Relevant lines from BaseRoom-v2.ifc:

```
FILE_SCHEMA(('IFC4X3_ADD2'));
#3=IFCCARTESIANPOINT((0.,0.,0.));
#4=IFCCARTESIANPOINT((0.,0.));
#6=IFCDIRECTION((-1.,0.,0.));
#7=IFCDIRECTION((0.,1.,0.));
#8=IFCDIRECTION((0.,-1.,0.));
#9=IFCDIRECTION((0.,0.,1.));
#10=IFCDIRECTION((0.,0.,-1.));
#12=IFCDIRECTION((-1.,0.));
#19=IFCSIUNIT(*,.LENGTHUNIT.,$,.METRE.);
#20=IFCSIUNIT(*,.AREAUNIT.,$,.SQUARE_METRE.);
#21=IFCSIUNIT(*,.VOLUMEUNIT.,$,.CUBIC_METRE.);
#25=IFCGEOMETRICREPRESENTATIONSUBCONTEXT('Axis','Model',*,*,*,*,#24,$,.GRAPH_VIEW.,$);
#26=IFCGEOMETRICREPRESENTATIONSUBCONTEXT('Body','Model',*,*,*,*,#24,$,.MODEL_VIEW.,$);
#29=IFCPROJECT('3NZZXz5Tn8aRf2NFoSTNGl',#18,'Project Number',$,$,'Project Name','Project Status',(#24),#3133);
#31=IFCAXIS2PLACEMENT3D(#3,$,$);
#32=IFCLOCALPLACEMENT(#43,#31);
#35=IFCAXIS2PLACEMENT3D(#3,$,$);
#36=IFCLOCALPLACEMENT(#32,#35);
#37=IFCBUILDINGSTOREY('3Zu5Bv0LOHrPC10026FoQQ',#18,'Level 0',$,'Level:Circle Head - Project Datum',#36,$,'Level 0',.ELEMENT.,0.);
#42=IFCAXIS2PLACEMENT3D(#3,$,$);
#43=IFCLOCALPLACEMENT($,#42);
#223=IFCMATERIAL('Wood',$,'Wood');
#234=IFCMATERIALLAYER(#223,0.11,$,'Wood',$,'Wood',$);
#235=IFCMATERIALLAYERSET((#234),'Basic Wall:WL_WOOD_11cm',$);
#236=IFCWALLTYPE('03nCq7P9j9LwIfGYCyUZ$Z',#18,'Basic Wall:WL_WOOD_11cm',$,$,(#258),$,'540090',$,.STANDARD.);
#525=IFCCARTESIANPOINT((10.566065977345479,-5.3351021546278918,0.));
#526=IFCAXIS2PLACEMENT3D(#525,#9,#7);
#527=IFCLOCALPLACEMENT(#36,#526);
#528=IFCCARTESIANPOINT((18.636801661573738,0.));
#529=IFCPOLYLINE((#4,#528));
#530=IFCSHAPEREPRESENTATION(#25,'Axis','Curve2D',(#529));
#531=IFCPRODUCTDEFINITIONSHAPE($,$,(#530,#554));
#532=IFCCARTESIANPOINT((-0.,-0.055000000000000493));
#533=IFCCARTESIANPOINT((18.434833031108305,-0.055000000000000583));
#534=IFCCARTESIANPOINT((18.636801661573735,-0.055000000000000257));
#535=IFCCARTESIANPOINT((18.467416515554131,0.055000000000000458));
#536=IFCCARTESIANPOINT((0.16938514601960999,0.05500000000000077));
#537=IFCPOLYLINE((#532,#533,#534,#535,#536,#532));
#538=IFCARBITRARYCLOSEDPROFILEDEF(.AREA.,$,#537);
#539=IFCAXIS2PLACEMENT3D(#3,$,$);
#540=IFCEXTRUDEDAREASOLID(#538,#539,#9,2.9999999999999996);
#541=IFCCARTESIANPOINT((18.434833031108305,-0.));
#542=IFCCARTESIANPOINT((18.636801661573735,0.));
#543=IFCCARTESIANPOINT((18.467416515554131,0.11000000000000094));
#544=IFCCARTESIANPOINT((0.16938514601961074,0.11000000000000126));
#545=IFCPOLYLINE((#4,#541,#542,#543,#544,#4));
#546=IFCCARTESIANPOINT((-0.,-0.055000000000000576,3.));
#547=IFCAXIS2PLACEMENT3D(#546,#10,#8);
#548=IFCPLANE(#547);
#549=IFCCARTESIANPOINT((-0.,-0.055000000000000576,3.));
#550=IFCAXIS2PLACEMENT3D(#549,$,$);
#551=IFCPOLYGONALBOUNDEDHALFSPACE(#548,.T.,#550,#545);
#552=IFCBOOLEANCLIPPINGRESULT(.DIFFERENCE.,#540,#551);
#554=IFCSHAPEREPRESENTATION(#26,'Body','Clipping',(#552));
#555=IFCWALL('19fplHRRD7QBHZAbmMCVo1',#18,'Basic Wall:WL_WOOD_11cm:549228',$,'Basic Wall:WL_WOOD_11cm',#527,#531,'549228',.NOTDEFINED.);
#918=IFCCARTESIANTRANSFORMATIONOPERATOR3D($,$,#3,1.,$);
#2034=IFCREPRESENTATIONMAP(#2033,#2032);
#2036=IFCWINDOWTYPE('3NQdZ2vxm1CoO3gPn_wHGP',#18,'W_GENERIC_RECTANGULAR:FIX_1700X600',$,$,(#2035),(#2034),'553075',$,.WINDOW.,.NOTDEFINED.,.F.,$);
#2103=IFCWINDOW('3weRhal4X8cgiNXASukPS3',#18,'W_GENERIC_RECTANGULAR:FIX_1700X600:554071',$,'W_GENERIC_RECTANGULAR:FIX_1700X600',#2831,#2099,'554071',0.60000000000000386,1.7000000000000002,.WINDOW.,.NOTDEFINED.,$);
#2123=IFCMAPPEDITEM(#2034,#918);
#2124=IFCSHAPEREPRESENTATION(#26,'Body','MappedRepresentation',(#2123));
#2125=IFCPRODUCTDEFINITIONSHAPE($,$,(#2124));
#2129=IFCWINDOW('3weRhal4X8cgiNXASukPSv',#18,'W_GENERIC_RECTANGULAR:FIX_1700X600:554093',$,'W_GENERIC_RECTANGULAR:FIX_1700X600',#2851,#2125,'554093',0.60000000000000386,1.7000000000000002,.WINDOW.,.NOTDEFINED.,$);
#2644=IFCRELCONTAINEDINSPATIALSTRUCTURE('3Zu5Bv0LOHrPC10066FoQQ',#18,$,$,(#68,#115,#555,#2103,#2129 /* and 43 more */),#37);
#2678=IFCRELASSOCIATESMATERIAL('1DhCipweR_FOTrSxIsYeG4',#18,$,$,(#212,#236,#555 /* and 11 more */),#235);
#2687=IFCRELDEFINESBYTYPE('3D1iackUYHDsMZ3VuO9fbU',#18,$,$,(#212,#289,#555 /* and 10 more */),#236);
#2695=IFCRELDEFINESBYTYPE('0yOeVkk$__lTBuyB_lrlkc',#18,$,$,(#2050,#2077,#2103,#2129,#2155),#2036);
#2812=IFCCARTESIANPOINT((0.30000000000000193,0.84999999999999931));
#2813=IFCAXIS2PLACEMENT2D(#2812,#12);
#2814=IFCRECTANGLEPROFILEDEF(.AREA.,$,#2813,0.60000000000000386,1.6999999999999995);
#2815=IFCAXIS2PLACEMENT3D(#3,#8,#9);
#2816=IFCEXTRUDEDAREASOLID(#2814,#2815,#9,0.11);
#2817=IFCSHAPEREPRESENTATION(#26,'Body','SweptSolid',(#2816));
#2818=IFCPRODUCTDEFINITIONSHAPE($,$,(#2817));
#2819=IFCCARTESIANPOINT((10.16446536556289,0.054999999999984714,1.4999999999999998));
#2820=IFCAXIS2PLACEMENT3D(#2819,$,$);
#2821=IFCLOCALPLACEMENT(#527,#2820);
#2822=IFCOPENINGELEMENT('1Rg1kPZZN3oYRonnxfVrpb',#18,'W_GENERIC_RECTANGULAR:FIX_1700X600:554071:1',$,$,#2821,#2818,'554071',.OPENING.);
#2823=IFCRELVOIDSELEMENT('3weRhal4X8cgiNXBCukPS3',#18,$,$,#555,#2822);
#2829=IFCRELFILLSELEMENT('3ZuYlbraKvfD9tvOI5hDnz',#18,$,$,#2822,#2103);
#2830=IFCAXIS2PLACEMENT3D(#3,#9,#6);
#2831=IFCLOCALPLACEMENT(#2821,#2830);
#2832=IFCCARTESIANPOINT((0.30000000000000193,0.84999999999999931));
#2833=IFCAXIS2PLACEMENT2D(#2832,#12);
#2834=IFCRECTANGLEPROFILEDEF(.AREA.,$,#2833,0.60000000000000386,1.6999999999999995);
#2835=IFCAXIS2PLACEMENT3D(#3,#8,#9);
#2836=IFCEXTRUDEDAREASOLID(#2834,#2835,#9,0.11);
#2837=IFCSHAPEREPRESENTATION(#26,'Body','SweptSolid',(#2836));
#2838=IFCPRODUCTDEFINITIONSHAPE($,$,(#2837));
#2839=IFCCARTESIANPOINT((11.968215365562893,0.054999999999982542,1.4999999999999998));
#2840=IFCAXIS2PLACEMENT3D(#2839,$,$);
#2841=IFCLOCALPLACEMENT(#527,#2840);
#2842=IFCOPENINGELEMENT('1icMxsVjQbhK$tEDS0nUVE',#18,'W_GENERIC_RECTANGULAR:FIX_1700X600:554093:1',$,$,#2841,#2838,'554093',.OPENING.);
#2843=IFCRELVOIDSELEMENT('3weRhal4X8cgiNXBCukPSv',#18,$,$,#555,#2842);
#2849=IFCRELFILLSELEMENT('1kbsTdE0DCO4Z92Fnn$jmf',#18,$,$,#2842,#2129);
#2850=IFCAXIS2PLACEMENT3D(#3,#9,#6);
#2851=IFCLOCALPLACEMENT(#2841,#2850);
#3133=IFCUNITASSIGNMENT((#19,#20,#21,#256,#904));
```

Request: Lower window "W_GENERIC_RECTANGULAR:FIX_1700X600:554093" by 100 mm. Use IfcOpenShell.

```python
import numpy as np
import ifcopenshell
import ifcopenshell.api.geometry
import ifcopenshell.util.placement
import ifcopenshell.util.unit

model = ifcopenshell.open("BaseRoom-v2.ifc")
unit_scale = ifcopenshell.util.unit.calculate_unit_scale(model)

window = model.by_guid("3weRhal4X8cgiNXASukPSv")
opening = window.FillsVoids[0].RelatingOpeningElement
dz = -0.1

shift = np.array([0.0, 0.0, dz])
# The window is placed relative to its opening, so it follows when the opening moves.
matrix = ifcopenshell.util.placement.get_local_placement(opening.ObjectPlacement)
matrix[:3, 3] += shift
ifcopenshell.api.geometry.edit_object_placement(
    model, product=opening, matrix=matrix, is_si=False, should_transform_children=True
)

print(f"moved by {dz * unit_scale:+.3f} m")

model.write("BaseRoom-v2_edited.ifc")
```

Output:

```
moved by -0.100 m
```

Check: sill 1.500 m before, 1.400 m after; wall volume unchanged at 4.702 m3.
